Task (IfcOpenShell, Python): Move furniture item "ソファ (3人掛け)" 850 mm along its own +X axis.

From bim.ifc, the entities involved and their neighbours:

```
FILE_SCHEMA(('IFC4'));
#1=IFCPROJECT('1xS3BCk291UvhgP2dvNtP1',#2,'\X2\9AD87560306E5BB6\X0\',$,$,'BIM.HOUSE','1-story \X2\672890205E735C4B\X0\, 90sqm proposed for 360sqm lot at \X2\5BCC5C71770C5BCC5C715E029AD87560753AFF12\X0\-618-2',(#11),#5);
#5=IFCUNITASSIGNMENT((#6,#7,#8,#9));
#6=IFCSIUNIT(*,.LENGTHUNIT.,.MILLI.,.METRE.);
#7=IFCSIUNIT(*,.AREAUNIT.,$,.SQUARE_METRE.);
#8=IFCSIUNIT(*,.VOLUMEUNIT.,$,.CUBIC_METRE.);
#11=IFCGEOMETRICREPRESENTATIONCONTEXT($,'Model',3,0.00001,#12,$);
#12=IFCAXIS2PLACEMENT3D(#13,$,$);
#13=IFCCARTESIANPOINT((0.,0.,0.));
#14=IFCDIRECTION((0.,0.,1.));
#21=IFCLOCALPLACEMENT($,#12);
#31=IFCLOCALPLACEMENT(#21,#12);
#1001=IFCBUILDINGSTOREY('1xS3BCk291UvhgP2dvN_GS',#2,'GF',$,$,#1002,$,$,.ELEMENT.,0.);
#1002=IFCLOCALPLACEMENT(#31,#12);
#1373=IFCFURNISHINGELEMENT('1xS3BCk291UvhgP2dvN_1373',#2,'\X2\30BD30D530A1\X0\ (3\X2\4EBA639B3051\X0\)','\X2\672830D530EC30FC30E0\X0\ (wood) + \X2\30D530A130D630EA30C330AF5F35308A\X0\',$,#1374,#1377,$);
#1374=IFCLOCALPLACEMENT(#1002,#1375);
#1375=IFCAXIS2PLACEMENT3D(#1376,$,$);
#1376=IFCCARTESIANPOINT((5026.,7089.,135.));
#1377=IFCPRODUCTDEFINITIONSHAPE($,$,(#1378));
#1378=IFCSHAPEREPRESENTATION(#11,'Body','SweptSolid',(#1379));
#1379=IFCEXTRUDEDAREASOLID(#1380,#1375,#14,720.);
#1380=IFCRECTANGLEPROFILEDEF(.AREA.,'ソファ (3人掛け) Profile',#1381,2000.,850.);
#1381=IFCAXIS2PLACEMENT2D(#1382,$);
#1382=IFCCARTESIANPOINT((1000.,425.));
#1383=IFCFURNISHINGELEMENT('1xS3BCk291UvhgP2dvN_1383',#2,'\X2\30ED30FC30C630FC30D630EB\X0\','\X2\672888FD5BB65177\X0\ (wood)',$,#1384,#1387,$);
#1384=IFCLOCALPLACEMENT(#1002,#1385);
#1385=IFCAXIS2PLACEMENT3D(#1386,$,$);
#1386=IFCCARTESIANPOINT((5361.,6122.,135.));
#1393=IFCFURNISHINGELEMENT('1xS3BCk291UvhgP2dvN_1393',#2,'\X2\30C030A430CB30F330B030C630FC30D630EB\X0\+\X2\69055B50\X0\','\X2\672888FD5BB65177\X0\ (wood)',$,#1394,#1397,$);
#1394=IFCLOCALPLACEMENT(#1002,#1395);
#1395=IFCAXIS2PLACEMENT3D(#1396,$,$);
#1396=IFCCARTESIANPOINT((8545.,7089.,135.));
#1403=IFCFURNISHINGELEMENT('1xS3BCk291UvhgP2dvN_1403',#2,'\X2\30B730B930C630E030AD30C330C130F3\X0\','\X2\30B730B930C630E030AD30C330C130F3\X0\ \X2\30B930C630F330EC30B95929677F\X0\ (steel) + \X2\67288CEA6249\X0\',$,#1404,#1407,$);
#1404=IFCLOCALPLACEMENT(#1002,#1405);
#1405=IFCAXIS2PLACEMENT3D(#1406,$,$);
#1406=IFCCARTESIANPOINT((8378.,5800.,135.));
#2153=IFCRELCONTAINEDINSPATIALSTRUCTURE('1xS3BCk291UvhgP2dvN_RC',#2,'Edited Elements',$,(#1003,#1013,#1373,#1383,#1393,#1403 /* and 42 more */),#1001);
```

```python
import ifcopenshell
import ifcopenshell.api.geometry
import ifcopenshell.util.placement

model = ifcopenshell.open("bim.ifc")

item = model.by_id(1373)
matrix = ifcopenshell.util.placement.get_local_placement(item.ObjectPlacement)
matrix[:3, 3] += matrix[:3, 0] * 850.0
ifcopenshell.api.geometry.edit_object_placement(model, product=item, matrix=matrix, is_si=False)

print(ifcopenshell.util.placement.get_local_placement(item.ObjectPlacement).round(3) + 0.0)

model.write("bim_edited.ifc")
```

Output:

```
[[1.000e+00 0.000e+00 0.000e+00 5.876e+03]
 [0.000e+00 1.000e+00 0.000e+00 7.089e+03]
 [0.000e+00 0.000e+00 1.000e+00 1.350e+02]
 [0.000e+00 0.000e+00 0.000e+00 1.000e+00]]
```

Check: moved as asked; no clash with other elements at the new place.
